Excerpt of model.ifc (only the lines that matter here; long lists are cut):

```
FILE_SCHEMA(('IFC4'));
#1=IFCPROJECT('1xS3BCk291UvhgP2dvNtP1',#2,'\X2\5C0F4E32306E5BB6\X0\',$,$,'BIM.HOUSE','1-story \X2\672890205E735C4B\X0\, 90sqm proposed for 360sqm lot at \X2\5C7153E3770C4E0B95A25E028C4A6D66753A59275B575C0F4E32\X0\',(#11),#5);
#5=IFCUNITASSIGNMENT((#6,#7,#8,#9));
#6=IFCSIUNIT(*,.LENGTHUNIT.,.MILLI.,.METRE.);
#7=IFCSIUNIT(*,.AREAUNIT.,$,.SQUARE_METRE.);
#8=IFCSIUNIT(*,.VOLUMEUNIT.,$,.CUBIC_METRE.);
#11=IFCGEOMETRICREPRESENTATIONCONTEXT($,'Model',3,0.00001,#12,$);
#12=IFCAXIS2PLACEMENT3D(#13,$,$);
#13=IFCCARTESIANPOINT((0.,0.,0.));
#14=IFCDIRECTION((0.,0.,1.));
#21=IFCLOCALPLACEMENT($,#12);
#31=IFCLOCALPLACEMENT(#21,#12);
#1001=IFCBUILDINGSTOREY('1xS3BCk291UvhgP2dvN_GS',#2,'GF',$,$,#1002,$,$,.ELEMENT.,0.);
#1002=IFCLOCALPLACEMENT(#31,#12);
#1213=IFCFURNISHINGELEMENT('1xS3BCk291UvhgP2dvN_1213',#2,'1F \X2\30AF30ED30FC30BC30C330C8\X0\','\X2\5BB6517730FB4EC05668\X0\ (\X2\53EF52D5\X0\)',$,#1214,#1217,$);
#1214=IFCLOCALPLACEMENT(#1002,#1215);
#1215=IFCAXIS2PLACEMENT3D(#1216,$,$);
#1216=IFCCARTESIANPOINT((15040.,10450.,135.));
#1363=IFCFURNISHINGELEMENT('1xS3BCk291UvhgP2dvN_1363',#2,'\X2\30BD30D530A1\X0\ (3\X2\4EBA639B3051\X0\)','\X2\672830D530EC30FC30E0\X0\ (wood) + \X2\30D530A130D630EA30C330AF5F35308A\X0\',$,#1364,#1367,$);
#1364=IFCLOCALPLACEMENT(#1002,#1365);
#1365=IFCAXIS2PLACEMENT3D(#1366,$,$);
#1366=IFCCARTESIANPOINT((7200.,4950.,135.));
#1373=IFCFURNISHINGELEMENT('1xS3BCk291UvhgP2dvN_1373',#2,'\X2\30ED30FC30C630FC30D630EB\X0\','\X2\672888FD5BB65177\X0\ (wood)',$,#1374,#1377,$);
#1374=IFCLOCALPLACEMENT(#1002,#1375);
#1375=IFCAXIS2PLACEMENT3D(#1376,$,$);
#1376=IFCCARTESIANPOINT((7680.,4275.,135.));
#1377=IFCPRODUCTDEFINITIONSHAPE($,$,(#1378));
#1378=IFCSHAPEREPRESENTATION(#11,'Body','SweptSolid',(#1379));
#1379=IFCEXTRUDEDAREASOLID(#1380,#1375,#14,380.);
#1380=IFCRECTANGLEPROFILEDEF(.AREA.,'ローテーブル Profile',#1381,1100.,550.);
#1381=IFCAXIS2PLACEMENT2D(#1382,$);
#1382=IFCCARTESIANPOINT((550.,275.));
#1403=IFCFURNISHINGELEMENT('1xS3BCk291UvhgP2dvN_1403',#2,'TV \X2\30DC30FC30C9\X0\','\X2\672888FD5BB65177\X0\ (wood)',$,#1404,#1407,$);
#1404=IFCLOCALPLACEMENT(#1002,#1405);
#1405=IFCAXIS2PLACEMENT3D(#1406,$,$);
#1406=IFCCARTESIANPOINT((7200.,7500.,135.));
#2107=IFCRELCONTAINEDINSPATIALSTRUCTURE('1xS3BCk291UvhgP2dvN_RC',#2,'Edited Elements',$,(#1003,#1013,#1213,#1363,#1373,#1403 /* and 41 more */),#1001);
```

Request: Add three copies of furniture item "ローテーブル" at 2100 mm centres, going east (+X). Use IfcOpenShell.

```python
import numpy as np
import ifcopenshell
import ifcopenshell.api.geometry
import ifcopenshell.api.root
import ifcopenshell.util.element
import ifcopenshell.util.placement
import ifcopenshell.util.unit

model = ifcopenshell.open("model.ifc")
unit_scale = ifcopenshell.util.unit.calculate_unit_scale(model)


def reuse_history(source, copy):
    """copy_class also copies each property set's owner history, people and application; keep the originals."""
    for rel in copy.IsDefinedBy:
        if rel.is_a("IfcRelDefinesByProperties") and (history := rel.RelatingPropertyDefinition.OwnerHistory):
            rel.RelatingPropertyDefinition.OwnerHistory = source.OwnerHistory
            ifcopenshell.util.element.remove_deep2(model, history)


source = model.by_guid("1xS3BCk291UvhgP2dvN_1373")
base = ifcopenshell.util.placement.get_local_placement(source.ObjectPlacement)
step = np.array([1.0, 0.0, 0.0]) * 2.1 / unit_scale

for i in range(1, 4):
    copy = ifcopenshell.api.root.copy_class(model, product=source)
    copy.Representation = ifcopenshell.util.element.copy_deep(
        model, source.Representation, exclude=["IfcGeometricRepresentationContext", "IfcRepresentationMap"]
    )
    reuse_history(source, copy)
    matrix = base.copy()
    matrix[:3, 3] += i * step
    print("added at", matrix[:3, 3].round(3) + 0.0)
    ifcopenshell.api.geometry.edit_object_placement(model, product=copy, matrix=matrix, is_si=False)

model.write("model_updated.ifc")
```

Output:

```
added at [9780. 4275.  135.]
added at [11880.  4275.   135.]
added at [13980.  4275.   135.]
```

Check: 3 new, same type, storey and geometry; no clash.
